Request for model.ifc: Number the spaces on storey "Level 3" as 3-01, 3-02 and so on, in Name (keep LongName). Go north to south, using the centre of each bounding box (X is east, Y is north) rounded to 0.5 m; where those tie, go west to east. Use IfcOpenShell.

First a look at what the model holds.

```python
import ifcopenshell
import ifcopenshell.util.element
import ifcopenshell.util.placement

model = ifcopenshell.open("model.ifc")
print(model.schema)
storey = next(s for s in model.by_type("IfcBuildingStorey") if s.Name == "Level 3")
spaces = [e for e in ifcopenshell.util.element.get_decomposition(storey) if e.is_a("IfcSpace")]
for e in sorted(spaces, key=lambda e: e.id()):
    origin = ifcopenshell.util.placement.get_local_placement(e.ObjectPlacement)[:3, 3]
    print(e.id(), e.Name, e.LongName, origin.round(2) + 0.0, sep=" | ")
```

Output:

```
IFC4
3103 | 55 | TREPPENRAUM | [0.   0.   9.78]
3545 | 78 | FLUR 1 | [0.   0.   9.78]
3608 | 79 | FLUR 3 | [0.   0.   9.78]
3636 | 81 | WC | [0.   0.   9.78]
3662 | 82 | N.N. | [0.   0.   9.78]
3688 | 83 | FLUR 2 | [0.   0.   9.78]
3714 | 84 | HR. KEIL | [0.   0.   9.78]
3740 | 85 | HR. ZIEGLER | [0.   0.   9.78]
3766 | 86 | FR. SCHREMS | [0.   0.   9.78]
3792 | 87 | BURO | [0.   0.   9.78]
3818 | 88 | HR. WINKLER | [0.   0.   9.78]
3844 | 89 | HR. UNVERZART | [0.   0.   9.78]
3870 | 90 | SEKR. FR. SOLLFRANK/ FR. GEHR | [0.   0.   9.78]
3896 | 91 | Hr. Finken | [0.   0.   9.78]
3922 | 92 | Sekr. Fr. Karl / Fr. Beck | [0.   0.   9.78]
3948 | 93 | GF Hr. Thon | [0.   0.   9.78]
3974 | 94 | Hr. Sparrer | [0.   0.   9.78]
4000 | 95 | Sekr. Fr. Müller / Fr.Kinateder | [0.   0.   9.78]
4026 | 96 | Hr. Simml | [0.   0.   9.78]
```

```python
import ifcopenshell
import ifcopenshell.geom
import ifcopenshell.util.element
import ifcopenshell.util.shape

model = ifcopenshell.open("model.ifc")
settings = ifcopenshell.geom.settings()
settings.set("use-world-coords", True)


def centre(element):
    shape = ifcopenshell.geom.create_shape(settings, element)
    return ifcopenshell.util.shape.get_bbox_centroid(shape.geometry)


storey = next(s for s in model.by_type("IfcBuildingStorey") if s.Name == "Level 3")
spaces = [e for e in ifcopenshell.util.element.get_decomposition(storey) if e.is_a("IfcSpace")]

# Insertion points can sit at a corner or the storey origin, so sort by the geometry (in metres).
centres = {e: centre(e) for e in spaces}
spaces.sort(key=lambda e: (-round(centres[e][1] / 0.5), centres[e][0]))

for i, e in enumerate(spaces, start=1):
    number = f"3-{i:02d}"
    e.Name = number
    print(e.id(), number)

model.write("model-out.ifc")
```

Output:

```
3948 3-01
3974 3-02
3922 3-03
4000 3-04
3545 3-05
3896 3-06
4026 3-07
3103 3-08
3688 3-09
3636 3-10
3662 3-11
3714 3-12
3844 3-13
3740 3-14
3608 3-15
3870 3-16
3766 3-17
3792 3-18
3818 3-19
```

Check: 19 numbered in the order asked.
